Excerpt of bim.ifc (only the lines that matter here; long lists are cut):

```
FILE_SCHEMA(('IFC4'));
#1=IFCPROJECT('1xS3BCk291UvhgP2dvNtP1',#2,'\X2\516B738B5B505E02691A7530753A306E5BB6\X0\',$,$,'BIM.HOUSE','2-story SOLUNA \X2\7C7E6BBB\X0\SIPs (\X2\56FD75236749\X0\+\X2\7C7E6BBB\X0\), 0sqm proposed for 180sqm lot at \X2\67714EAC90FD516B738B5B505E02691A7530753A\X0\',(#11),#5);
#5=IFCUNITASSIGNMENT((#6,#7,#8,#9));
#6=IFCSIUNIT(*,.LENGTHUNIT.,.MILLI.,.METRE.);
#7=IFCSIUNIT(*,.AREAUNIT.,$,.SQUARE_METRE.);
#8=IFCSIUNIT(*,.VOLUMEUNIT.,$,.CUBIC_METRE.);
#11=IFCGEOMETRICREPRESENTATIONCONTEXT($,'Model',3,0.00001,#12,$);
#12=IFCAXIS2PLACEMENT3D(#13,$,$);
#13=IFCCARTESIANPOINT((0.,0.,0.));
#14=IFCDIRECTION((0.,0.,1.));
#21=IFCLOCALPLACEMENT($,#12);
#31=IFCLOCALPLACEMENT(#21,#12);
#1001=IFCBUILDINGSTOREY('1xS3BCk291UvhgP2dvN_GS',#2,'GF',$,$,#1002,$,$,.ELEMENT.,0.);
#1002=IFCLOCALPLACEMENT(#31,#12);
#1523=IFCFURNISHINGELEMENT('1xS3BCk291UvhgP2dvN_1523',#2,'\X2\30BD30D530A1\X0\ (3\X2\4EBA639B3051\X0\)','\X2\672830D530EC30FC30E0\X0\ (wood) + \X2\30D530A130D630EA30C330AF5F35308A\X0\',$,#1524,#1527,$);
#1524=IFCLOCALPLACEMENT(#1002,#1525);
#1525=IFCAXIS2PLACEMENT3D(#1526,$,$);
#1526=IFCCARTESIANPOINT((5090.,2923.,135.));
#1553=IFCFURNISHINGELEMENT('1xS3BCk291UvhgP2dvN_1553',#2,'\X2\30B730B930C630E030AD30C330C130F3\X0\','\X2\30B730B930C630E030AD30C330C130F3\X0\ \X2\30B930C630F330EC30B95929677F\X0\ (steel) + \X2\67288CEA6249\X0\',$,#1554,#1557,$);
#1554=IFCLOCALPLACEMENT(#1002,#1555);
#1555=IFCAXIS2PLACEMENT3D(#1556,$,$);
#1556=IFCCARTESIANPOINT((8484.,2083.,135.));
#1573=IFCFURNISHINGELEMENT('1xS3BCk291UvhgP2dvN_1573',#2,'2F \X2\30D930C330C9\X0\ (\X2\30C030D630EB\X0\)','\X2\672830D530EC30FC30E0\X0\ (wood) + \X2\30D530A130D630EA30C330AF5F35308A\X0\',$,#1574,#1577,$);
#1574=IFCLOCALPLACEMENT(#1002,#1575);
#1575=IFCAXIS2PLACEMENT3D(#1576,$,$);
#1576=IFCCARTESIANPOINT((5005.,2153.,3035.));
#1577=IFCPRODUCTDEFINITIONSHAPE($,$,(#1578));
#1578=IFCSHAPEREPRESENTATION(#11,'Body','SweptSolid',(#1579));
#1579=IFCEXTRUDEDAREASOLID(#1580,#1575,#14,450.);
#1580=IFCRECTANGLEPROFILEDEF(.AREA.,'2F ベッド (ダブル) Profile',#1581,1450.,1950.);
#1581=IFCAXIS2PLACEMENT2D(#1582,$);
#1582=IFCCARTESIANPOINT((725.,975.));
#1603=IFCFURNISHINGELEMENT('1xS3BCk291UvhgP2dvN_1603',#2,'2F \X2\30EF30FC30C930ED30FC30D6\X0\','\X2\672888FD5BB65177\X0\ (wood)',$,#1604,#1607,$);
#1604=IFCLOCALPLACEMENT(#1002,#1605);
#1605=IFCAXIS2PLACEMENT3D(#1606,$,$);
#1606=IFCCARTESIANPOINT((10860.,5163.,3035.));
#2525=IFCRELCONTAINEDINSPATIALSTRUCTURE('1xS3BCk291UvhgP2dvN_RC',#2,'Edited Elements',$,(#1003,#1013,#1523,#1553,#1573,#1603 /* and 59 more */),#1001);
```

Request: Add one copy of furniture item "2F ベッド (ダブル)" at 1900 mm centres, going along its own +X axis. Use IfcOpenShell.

```python
import ifcopenshell
import ifcopenshell.api.geometry
import ifcopenshell.api.root
import ifcopenshell.util.element
import ifcopenshell.util.placement
import ifcopenshell.util.unit

model = ifcopenshell.open("bim.ifc")
unit_scale = ifcopenshell.util.unit.calculate_unit_scale(model)


def reuse_history(source, copy):
    """copy_class also copies each property set's owner history, people and application; keep the originals."""
    for rel in copy.IsDefinedBy:
        if rel.is_a("IfcRelDefinesByProperties") and (history := rel.RelatingPropertyDefinition.OwnerHistory):
            rel.RelatingPropertyDefinition.OwnerHistory = source.OwnerHistory
            ifcopenshell.util.element.remove_deep2(model, history)


source = model.by_id(1573)
base = ifcopenshell.util.placement.get_local_placement(source.ObjectPlacement)
step = base[:3, 0] * 1.9 / unit_scale

for i in range(1, 2):
    copy = ifcopenshell.api.root.copy_class(model, product=source)
    copy.Representation = ifcopenshell.util.element.copy_deep(
        model, source.Representation, exclude=["IfcGeometricRepresentationContext", "IfcRepresentationMap"]
    )
    reuse_history(source, copy)
    matrix = base.copy()
    matrix[:3, 3] += i * step
    print("added at", matrix[:3, 3].round(3) + 0.0)
    ifcopenshell.api.geometry.edit_object_placement(model, product=copy, matrix=matrix, is_si=False)

model.write("bim_updated.ifc")
```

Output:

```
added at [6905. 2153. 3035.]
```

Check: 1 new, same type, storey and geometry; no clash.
